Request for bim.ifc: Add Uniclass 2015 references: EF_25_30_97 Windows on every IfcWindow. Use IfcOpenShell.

First a look at what the model holds.

```python
import ifcopenshell

model = ifcopenshell.open("bim.ifc")
print(model.schema)
print("classifications:", [c.Name for c in model.by_type("IfcClassification")])
for ifc_class in ("IfcDoor", "IfcRoof", "IfcStair", "IfcWall", "IfcWindow"):
    print(ifc_class, len(model.by_type(ifc_class)))
```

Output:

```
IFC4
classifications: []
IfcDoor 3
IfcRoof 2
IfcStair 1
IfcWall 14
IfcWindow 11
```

```python
import ifcopenshell
import ifcopenshell.api.classification

model = ifcopenshell.open("bim.ifc")

system = ifcopenshell.api.classification.add_classification(model, classification="Uniclass 2015")

codes = {
    "IfcWindow": ("EF_25_30_97", "Windows"),
}
for ifc_class, (code, name) in codes.items():
    products = model.by_type(ifc_class)
    ifcopenshell.api.classification.add_reference(
        model, products=products, classification=system, identification=code, name=name
    )
    print(code, len(products))

model.write("bim_v2.ifc")
```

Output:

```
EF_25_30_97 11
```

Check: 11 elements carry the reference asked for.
